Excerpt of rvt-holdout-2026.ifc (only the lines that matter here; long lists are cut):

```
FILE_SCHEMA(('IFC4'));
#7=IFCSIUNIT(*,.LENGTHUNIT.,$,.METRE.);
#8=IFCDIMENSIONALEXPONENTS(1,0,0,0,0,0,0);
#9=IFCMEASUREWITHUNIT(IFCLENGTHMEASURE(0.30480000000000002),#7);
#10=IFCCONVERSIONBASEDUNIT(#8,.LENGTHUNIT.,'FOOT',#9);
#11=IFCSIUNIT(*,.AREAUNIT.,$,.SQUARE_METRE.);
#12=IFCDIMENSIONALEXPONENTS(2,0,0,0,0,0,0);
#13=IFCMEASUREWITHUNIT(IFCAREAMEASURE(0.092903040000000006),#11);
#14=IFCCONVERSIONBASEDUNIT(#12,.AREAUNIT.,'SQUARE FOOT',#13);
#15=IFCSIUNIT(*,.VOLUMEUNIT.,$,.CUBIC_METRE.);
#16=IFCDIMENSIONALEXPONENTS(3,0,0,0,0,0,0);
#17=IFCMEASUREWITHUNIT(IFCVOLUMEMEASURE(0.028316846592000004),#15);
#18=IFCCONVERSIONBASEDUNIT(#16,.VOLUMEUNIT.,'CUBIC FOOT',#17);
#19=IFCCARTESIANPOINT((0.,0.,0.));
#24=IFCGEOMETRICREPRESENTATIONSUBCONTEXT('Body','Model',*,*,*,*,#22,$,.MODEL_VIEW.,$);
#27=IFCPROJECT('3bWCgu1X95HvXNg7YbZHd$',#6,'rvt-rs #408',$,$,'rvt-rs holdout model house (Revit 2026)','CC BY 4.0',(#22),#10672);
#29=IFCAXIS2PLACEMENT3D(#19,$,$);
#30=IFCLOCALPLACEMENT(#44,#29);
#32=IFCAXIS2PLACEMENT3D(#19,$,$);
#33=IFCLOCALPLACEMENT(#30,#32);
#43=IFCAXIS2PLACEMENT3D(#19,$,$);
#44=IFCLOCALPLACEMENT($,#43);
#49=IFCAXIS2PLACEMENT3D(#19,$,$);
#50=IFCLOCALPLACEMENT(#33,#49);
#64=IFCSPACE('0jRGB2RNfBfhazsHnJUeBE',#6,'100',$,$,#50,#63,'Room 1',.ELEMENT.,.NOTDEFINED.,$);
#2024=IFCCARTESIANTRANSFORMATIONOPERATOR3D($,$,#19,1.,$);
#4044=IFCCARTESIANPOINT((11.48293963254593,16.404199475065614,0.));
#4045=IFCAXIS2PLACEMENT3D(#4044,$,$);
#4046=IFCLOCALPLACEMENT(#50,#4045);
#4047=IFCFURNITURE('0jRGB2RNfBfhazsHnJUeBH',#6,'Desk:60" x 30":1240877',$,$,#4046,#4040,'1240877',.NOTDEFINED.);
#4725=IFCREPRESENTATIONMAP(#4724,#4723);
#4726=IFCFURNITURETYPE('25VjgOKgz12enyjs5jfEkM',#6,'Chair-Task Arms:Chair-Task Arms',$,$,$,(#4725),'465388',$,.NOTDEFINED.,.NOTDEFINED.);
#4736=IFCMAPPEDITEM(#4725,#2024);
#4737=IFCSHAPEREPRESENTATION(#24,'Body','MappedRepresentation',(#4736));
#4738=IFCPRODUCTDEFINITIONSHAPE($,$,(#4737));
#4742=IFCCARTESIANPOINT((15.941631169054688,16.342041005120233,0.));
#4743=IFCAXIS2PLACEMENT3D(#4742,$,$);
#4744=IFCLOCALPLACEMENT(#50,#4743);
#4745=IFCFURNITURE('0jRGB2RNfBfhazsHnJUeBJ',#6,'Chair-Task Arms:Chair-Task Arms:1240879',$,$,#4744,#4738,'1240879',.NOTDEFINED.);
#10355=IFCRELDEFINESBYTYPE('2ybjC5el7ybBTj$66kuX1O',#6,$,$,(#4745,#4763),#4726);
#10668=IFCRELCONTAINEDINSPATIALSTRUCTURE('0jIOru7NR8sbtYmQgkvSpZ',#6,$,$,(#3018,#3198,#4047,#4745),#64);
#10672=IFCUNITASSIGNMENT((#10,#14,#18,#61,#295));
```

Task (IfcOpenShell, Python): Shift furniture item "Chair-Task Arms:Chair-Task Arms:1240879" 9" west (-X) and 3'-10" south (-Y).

```python
import ifcopenshell
import ifcopenshell.api.geometry
import ifcopenshell.util.placement
import ifcopenshell.util.unit

model = ifcopenshell.open("rvt-holdout-2026.ifc")
unit_scale = ifcopenshell.util.unit.calculate_unit_scale(model)

item = model.by_guid("0jRGB2RNfBfhazsHnJUeBJ")
matrix = ifcopenshell.util.placement.get_local_placement(item.ObjectPlacement)
matrix[0, 3] -= 9 * 0.0254 / unit_scale
matrix[1, 3] -= 46 * 0.0254 / unit_scale
ifcopenshell.api.geometry.edit_object_placement(model, product=item, matrix=matrix, is_si=False)

print(ifcopenshell.util.placement.get_local_placement(item.ObjectPlacement).round(3) + 0.0)

model.write("rvt-holdout-2026_edited.ifc")
```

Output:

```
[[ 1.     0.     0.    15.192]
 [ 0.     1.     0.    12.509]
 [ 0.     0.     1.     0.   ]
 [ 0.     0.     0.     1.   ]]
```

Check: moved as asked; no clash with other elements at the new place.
